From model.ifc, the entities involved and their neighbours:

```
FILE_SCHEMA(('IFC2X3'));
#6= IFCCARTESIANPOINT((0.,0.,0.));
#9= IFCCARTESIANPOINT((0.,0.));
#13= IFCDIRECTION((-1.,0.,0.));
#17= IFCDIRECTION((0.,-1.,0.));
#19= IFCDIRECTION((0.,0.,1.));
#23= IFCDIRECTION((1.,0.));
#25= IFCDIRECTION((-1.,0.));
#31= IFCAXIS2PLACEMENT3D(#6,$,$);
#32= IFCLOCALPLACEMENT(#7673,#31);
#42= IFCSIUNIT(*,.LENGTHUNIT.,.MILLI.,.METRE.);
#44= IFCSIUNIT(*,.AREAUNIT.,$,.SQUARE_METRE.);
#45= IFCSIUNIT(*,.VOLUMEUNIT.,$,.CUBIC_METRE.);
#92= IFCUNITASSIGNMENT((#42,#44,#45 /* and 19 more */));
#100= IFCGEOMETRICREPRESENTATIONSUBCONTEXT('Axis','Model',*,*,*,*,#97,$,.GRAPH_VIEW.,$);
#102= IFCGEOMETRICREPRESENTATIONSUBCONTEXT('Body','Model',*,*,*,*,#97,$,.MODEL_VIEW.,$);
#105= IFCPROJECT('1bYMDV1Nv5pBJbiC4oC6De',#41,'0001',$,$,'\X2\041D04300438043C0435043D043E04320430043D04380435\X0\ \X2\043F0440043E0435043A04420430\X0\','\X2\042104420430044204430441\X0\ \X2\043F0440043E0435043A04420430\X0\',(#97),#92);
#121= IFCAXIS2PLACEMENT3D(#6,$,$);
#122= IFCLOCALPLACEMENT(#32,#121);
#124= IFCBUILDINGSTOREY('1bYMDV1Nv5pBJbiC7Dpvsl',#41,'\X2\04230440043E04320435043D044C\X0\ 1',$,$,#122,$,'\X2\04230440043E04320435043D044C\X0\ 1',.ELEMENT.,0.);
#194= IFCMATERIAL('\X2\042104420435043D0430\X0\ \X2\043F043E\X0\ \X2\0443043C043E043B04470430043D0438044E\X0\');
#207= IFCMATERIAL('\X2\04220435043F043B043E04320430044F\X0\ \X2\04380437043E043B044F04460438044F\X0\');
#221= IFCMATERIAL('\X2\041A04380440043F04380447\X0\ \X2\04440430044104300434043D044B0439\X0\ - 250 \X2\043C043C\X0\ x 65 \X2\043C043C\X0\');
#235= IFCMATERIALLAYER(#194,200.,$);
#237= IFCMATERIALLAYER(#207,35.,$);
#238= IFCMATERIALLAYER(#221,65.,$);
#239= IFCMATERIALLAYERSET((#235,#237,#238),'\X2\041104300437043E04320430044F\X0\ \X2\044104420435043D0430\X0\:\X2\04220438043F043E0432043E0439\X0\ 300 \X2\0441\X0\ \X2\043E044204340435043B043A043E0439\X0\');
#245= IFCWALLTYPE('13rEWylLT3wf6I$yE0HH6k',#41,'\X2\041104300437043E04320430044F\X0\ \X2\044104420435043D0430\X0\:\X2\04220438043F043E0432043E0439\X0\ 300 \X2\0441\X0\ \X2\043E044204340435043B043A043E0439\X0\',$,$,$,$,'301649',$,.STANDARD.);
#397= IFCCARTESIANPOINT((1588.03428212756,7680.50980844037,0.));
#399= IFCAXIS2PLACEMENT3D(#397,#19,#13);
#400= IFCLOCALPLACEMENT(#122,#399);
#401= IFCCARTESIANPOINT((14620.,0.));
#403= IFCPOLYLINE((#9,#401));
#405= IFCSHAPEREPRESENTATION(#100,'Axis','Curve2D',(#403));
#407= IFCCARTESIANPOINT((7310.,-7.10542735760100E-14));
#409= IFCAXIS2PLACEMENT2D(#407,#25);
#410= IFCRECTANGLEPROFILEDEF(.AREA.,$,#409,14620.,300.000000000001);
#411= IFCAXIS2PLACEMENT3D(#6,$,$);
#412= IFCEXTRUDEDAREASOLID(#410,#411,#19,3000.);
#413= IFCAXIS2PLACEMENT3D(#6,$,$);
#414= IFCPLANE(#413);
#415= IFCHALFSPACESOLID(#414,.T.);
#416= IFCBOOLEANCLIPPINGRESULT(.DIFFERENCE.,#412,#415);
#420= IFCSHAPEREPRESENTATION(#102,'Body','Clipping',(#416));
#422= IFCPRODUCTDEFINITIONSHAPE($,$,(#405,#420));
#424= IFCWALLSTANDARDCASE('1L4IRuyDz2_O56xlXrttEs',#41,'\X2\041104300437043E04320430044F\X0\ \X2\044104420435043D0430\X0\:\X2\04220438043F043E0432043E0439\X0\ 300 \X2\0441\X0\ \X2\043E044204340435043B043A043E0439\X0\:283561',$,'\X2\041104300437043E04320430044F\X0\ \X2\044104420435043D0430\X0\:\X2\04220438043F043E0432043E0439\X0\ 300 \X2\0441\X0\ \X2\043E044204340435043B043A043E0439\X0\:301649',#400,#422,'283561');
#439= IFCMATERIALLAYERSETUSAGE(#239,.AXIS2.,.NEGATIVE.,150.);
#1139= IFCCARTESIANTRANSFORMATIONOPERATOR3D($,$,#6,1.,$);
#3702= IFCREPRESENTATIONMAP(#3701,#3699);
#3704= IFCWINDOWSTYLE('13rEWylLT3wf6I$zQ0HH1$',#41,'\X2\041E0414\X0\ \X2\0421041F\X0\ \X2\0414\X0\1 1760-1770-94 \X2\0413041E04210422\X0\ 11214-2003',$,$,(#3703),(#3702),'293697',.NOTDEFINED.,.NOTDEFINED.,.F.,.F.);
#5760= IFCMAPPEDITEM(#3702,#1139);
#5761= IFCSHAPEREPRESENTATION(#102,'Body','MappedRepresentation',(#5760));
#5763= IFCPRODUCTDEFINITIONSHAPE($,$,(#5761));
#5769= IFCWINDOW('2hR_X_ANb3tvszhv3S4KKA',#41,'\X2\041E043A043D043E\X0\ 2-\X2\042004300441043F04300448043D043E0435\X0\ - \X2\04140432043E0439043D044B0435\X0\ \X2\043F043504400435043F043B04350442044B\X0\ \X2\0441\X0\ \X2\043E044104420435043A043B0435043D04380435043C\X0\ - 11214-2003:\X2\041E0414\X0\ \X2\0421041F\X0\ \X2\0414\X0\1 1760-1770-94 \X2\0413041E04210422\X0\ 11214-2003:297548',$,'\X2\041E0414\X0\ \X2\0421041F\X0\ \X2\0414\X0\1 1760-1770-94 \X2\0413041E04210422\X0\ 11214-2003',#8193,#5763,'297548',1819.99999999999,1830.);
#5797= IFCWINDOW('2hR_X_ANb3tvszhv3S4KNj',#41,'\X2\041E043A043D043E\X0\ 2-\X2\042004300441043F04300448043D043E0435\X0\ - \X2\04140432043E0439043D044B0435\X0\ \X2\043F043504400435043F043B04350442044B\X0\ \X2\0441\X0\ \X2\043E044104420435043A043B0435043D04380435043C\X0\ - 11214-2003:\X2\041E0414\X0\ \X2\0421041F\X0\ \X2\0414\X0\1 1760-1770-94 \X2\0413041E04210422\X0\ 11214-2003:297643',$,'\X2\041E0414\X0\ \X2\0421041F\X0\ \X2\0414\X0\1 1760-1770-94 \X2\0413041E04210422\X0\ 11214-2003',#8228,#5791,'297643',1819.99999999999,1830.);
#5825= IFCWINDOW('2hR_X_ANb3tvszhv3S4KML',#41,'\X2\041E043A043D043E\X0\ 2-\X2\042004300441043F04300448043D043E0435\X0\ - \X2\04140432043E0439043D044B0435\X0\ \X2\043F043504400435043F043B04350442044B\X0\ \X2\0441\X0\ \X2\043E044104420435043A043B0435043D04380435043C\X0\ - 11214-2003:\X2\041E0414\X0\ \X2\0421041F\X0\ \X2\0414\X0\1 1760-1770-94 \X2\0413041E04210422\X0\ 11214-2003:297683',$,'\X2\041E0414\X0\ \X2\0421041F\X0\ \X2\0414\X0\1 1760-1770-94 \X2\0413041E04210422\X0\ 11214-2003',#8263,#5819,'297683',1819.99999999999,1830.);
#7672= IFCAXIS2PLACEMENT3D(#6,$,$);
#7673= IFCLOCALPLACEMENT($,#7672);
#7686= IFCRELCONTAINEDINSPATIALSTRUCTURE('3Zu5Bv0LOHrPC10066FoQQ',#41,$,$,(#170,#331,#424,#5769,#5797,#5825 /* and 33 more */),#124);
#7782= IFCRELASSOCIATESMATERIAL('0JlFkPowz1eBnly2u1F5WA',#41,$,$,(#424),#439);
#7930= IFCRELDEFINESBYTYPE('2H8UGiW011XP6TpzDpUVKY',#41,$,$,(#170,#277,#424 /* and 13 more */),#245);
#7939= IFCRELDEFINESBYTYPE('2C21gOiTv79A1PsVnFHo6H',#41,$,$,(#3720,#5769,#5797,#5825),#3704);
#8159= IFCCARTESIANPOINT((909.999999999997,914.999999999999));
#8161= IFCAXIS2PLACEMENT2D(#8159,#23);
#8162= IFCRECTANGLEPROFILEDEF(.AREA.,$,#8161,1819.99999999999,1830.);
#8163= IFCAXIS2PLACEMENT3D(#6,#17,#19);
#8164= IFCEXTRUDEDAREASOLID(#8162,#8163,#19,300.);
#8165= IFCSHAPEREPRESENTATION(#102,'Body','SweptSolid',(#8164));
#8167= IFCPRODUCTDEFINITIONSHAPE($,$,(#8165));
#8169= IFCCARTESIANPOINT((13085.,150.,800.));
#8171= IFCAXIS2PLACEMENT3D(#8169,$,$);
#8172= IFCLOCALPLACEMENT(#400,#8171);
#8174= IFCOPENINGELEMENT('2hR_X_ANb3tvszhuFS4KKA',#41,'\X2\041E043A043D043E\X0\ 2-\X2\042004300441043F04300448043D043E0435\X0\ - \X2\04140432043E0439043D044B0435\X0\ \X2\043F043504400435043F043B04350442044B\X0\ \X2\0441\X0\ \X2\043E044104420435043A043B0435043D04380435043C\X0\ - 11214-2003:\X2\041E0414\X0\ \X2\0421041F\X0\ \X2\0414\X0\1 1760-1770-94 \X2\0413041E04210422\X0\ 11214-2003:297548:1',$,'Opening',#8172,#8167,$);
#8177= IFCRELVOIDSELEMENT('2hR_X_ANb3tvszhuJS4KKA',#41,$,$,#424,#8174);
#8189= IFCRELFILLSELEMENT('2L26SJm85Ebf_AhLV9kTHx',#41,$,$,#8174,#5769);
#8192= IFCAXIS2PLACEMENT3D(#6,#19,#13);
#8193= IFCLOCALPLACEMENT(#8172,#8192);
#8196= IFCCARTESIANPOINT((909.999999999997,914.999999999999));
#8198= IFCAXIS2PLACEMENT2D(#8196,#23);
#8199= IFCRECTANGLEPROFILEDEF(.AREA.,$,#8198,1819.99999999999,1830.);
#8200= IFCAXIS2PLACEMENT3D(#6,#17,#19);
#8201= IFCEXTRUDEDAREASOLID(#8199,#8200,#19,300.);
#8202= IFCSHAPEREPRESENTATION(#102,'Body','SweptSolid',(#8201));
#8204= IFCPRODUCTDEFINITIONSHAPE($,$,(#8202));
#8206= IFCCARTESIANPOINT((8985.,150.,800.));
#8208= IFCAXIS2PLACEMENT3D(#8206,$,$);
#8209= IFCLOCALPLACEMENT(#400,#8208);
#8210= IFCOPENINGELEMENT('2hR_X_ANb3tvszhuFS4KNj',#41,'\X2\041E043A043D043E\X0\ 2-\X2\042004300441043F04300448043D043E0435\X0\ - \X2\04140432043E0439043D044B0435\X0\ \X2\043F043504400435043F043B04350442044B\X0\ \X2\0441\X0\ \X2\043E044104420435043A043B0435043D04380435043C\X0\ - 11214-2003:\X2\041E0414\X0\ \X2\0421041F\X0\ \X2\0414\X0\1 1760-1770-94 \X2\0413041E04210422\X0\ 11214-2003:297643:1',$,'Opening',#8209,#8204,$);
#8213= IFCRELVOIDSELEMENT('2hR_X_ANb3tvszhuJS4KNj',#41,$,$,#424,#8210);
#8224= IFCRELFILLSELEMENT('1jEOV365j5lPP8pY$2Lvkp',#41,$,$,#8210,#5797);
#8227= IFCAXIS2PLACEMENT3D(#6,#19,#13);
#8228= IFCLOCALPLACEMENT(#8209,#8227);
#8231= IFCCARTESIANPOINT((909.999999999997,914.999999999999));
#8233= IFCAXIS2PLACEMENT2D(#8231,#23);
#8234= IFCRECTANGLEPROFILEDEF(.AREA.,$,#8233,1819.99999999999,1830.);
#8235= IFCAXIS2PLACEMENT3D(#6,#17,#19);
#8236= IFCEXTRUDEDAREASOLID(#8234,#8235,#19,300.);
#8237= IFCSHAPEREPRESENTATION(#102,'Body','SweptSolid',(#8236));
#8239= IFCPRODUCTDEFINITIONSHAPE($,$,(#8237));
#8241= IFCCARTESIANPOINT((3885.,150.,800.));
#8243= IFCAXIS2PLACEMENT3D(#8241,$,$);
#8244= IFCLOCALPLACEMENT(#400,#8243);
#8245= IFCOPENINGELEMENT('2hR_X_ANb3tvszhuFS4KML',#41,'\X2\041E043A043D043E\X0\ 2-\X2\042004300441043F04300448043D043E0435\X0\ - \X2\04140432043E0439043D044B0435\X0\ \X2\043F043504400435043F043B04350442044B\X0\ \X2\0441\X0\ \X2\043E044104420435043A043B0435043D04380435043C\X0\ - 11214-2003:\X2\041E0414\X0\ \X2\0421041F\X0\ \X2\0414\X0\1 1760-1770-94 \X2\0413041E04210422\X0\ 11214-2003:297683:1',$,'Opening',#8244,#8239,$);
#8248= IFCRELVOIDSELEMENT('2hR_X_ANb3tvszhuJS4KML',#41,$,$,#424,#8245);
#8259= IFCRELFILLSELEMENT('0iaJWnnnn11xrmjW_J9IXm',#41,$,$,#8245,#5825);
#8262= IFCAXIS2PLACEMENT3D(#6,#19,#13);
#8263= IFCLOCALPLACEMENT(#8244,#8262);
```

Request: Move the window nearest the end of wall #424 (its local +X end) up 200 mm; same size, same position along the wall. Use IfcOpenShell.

```python
import numpy as np
import ifcopenshell
import ifcopenshell.api.geometry
import ifcopenshell.util.placement
import ifcopenshell.util.unit

model = ifcopenshell.open("model.ifc")
unit_scale = ifcopenshell.util.unit.calculate_unit_scale(model)

window = model.by_guid("2hR_X_ANb3tvszhv3S4KKA")
opening = window.FillsVoids[0].RelatingOpeningElement
dz = 200.0

shift = np.array([0.0, 0.0, dz])
# The window is placed relative to its opening, so it follows when the opening moves.
matrix = ifcopenshell.util.placement.get_local_placement(opening.ObjectPlacement)
matrix[:3, 3] += shift
ifcopenshell.api.geometry.edit_object_placement(
    model, product=opening, matrix=matrix, is_si=False, should_transform_children=True
)

print(f"moved by {dz * unit_scale:+.3f} m")

model.write("model_v2.ifc")
```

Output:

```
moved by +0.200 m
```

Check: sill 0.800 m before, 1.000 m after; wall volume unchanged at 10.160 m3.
